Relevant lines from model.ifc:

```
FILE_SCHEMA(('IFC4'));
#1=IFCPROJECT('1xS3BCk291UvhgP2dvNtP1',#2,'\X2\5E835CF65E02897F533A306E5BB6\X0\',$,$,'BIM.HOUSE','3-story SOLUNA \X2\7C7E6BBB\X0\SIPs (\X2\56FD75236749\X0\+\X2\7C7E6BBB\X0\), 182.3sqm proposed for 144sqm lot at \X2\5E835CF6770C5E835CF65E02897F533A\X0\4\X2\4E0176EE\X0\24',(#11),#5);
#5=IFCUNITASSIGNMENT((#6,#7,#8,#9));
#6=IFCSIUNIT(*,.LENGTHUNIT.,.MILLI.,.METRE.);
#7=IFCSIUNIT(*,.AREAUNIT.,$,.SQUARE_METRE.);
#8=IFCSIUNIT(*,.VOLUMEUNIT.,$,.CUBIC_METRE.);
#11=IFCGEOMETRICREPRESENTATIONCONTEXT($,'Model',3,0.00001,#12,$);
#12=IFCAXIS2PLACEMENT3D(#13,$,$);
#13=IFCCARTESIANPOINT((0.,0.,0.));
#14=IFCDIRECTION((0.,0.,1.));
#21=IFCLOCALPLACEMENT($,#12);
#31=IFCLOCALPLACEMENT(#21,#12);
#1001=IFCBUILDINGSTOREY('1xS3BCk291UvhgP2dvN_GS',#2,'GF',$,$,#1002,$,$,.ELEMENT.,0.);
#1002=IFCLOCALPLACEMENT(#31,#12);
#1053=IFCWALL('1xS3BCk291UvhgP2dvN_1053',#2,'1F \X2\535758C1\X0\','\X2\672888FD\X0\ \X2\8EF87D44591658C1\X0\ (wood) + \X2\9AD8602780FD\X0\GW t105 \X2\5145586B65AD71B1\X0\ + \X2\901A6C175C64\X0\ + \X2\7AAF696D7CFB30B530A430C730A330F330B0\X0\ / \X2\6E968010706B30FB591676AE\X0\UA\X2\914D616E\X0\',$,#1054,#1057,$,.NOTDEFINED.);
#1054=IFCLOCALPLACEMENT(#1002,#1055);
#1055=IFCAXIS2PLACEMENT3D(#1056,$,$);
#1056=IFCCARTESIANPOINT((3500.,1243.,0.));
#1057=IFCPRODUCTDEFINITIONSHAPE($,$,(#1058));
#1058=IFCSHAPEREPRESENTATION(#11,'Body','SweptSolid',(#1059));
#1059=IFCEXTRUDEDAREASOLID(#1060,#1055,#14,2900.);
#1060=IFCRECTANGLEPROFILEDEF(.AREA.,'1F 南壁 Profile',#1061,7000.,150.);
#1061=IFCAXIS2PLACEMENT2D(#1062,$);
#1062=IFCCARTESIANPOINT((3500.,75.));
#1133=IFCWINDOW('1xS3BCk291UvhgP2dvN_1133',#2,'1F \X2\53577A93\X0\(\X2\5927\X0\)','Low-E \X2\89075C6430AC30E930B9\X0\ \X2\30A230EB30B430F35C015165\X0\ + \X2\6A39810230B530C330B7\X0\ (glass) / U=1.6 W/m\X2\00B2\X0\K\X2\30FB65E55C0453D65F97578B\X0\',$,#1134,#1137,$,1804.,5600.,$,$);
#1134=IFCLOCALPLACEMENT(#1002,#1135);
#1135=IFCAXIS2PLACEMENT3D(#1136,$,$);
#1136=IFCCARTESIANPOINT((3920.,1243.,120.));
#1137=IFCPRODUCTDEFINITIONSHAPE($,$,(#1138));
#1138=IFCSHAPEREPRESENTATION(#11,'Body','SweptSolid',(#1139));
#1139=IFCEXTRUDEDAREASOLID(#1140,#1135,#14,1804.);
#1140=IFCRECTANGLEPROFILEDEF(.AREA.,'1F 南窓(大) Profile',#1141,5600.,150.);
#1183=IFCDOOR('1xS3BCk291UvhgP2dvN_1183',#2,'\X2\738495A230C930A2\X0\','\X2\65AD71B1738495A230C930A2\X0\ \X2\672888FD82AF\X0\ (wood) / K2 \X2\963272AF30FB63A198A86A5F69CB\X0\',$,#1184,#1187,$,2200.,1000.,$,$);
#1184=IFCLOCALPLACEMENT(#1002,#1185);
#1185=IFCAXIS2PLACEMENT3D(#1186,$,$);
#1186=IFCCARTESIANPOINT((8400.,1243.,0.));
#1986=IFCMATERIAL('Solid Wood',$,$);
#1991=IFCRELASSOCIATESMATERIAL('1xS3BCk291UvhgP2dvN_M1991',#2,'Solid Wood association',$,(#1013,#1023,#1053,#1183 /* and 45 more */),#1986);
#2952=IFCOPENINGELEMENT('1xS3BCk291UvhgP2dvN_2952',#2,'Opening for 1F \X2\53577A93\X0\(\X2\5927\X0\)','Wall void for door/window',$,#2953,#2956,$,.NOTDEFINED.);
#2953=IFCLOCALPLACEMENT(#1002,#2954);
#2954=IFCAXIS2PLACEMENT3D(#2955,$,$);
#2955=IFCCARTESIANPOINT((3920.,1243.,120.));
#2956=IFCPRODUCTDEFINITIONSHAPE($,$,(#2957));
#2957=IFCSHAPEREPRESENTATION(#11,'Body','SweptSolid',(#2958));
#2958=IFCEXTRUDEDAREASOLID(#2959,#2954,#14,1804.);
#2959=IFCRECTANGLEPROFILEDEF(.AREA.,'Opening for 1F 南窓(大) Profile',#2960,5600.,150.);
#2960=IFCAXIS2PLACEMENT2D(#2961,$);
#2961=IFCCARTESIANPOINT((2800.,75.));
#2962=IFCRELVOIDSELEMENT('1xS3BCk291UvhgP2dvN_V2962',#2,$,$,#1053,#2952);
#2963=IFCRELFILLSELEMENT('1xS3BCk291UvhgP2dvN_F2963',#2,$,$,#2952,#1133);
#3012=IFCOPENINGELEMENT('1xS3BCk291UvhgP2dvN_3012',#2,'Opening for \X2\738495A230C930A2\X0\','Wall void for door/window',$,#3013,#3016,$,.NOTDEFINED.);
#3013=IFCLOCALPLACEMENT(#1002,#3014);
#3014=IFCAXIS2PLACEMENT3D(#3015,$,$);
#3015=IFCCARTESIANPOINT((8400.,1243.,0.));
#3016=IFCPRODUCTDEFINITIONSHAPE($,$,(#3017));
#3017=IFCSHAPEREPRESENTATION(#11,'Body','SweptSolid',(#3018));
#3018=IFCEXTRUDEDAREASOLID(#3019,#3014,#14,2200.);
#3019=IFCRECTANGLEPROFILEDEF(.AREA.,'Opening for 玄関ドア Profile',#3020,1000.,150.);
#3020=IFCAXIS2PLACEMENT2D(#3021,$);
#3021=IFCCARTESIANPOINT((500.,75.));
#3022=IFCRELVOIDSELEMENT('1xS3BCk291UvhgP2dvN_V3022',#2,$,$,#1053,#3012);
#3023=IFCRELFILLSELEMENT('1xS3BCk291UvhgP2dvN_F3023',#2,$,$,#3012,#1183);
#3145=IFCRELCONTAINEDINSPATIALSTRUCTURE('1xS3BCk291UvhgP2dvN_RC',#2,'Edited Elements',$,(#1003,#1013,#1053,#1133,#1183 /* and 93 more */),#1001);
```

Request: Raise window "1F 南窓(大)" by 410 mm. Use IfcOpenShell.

```python
import numpy as np
import ifcopenshell
import ifcopenshell.api.geometry
import ifcopenshell.util.placement
import ifcopenshell.util.unit

model = ifcopenshell.open("model.ifc")
unit_scale = ifcopenshell.util.unit.calculate_unit_scale(model)

window = model.by_guid("1xS3BCk291UvhgP2dvN_1133")
opening = window.FillsVoids[0].RelatingOpeningElement
dz = 410.0

shift = np.array([0.0, 0.0, dz])
# The window is not placed relative to its opening, so move both.
for product in (opening, window):
    matrix = ifcopenshell.util.placement.get_local_placement(product.ObjectPlacement)
    matrix[:3, 3] += shift
    ifcopenshell.api.geometry.edit_object_placement(model, product=product, matrix=matrix, is_si=False)

print(f"moved by {dz * unit_scale:+.3f} m")

model.write("model_v2.ifc")
```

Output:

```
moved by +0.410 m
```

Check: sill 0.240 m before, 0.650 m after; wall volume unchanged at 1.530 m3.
